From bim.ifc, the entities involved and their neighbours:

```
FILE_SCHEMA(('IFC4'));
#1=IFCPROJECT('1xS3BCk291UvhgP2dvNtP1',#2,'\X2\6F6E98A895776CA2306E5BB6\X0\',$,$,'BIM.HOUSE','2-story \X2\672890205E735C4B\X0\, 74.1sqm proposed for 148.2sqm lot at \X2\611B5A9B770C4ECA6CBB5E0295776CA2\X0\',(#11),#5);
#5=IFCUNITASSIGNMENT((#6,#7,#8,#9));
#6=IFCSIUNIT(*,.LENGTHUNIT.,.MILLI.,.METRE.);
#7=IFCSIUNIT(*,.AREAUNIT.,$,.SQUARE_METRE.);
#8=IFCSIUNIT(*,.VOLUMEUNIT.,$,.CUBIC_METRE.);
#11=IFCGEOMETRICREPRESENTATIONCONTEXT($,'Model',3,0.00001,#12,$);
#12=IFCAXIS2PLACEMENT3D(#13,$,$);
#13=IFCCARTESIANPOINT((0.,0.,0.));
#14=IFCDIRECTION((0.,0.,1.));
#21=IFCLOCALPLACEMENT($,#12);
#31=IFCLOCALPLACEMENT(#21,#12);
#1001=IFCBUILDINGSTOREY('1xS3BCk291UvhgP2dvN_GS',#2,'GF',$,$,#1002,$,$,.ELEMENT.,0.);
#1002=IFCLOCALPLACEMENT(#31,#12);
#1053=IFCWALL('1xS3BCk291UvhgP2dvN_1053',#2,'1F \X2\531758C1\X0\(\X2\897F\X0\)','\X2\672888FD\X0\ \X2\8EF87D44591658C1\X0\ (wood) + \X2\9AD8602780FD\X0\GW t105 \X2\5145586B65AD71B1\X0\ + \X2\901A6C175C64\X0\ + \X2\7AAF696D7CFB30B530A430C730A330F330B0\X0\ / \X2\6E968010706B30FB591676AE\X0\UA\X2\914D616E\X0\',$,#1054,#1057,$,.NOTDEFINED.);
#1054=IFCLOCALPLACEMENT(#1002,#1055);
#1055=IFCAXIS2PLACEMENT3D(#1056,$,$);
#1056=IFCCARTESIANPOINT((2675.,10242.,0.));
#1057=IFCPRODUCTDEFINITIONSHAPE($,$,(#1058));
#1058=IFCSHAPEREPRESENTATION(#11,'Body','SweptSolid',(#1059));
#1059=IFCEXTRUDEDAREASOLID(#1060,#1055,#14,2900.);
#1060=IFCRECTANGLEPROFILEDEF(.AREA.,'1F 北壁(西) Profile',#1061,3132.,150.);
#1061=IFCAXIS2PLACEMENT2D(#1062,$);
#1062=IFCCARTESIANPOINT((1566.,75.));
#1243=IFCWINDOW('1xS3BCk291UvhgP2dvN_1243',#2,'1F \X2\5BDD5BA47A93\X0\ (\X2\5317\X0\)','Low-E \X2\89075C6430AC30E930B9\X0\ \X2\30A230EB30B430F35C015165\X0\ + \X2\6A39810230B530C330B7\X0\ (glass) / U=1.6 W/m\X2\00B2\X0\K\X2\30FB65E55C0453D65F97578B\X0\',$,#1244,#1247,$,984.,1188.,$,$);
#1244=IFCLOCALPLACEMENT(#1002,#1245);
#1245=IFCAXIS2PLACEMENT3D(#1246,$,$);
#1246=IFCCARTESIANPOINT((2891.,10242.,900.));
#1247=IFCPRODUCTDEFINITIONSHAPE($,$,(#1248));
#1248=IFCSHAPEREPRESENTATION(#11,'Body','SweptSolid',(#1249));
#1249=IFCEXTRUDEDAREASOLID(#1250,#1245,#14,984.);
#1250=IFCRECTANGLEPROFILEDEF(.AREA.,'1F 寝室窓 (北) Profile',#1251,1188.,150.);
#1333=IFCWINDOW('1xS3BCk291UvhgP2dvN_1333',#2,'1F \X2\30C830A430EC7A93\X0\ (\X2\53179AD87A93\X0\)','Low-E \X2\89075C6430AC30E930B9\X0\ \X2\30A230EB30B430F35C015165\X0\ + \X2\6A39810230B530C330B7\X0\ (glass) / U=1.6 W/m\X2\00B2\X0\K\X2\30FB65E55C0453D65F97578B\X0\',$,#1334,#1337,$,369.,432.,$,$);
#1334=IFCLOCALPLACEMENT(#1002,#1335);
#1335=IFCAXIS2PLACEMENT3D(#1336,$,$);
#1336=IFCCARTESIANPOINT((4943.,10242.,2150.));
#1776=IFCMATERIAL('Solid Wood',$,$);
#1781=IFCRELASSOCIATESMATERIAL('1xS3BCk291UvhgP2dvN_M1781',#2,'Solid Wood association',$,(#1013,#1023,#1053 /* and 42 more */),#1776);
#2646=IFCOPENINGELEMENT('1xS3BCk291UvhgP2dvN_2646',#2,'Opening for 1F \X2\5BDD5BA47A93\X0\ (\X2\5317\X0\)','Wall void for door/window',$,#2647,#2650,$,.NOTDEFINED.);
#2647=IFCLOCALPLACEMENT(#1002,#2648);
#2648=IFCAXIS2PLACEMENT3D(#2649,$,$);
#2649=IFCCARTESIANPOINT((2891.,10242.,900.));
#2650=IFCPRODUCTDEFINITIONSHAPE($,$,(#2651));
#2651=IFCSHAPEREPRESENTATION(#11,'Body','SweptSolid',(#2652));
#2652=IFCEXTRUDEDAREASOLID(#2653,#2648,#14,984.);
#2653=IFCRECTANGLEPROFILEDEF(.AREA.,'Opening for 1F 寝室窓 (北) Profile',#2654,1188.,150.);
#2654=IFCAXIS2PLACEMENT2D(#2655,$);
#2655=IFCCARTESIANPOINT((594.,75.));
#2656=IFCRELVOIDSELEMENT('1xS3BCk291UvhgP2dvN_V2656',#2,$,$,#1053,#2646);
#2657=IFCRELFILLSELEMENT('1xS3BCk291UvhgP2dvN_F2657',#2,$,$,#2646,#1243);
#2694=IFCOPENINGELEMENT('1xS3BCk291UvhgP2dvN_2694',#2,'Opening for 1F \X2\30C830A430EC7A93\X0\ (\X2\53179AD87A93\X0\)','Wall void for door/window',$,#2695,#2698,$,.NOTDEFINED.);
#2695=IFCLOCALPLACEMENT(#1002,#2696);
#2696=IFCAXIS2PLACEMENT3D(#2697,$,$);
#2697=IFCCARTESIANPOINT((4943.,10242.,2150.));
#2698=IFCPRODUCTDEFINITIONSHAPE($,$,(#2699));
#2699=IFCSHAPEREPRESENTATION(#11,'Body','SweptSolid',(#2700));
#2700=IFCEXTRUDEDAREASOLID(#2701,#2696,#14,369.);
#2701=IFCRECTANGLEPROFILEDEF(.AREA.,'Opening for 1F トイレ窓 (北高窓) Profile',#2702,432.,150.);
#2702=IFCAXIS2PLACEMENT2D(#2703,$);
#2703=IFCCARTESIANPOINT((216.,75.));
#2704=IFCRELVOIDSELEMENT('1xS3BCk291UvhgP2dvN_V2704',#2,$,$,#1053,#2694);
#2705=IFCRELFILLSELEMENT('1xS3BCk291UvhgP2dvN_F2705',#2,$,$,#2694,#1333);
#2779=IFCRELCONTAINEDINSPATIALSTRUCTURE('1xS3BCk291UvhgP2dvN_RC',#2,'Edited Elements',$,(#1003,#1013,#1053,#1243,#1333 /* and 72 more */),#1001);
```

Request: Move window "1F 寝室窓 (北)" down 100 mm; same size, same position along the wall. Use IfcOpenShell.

```python
import numpy as np
import ifcopenshell
import ifcopenshell.api.geometry
import ifcopenshell.util.placement
import ifcopenshell.util.unit

model = ifcopenshell.open("bim.ifc")
unit_scale = ifcopenshell.util.unit.calculate_unit_scale(model)

window = model.by_guid("1xS3BCk291UvhgP2dvN_1243")
opening = window.FillsVoids[0].RelatingOpeningElement
dz = -0.1 / unit_scale

shift = np.array([0.0, 0.0, dz])
# The window is not placed relative to its opening, so move both.
for product in (opening, window):
    matrix = ifcopenshell.util.placement.get_local_placement(product.ObjectPlacement)
    matrix[:3, 3] += shift
    ifcopenshell.api.geometry.edit_object_placement(model, product=product, matrix=matrix, is_si=False)

print(f"moved by {dz * unit_scale:+.3f} m")

model.write("bim-out.ifc")
```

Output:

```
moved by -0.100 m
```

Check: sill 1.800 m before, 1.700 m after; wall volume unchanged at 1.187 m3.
